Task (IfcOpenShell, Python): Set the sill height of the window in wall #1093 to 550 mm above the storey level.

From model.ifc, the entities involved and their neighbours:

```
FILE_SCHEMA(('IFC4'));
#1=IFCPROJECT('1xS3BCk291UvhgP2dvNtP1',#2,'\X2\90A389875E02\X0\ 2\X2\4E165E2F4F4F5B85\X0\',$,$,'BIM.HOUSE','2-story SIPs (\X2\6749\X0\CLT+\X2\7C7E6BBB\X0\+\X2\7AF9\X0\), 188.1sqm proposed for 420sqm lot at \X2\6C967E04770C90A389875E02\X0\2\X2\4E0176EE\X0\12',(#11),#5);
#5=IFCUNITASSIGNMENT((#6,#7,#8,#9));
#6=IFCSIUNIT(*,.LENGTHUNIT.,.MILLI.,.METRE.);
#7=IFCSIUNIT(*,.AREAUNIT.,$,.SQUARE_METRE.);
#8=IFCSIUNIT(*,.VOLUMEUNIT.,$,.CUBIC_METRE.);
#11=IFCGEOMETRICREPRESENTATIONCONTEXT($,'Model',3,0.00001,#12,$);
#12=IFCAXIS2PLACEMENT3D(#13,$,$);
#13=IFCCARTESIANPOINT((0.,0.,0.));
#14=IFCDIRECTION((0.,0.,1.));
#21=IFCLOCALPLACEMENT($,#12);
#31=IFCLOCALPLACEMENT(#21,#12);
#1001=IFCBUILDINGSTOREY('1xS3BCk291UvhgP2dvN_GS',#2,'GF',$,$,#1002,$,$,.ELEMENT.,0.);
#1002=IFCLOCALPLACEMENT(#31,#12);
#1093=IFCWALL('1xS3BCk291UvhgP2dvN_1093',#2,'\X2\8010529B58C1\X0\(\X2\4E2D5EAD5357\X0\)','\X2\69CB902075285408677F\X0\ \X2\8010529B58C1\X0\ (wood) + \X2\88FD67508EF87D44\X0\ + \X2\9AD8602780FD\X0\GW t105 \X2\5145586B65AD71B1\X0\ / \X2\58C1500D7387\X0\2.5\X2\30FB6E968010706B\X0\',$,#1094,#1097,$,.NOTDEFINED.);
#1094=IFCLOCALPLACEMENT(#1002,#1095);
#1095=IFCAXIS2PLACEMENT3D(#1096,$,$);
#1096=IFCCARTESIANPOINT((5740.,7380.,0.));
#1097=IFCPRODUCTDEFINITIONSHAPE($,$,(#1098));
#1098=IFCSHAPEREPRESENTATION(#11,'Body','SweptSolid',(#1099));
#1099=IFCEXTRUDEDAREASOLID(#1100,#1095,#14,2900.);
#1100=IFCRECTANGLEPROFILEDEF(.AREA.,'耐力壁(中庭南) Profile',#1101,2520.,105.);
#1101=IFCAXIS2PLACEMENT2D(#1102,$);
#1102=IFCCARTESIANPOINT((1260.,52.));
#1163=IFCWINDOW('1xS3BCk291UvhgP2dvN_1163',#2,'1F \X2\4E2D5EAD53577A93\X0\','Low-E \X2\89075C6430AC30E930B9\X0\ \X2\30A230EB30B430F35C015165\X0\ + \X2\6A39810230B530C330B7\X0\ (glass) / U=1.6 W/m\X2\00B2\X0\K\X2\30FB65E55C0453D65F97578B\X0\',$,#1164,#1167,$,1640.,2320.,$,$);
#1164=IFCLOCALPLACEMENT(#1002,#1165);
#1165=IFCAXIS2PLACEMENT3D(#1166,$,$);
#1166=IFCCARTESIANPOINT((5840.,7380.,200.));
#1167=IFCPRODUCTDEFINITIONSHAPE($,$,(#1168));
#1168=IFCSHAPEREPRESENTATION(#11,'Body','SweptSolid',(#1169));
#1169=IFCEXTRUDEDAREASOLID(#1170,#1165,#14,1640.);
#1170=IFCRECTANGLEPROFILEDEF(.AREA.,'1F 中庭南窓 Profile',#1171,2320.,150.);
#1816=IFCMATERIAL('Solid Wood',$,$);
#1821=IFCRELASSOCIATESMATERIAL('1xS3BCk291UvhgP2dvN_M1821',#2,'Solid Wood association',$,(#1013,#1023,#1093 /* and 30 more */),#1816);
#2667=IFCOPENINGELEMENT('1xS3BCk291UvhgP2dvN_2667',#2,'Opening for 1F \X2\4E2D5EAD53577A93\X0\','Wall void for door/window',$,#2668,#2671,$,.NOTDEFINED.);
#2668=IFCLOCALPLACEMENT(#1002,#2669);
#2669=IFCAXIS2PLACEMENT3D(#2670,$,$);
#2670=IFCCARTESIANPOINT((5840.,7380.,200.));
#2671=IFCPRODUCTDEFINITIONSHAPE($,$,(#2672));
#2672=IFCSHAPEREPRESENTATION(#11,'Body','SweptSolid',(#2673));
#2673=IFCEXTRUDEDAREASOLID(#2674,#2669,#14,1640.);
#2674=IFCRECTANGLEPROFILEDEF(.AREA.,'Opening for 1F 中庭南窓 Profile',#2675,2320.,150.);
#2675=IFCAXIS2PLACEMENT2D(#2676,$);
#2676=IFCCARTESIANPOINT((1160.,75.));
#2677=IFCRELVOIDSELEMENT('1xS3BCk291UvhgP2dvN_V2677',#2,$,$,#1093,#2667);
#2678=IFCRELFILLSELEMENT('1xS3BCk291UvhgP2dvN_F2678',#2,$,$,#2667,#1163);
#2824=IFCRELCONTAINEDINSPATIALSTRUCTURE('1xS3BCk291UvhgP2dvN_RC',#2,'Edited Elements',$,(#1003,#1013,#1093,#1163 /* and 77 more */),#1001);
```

```python
import numpy as np
import ifcopenshell
import ifcopenshell.api.geometry
import ifcopenshell.geom
import ifcopenshell.util.element
import ifcopenshell.util.placement
import ifcopenshell.util.shape
import ifcopenshell.util.unit

model = ifcopenshell.open("model.ifc")
unit_scale = ifcopenshell.util.unit.calculate_unit_scale(model)

window = model.by_guid("1xS3BCk291UvhgP2dvN_1163")
opening = window.FillsVoids[0].RelatingOpeningElement
storey = ifcopenshell.util.element.get_container(window, ifc_class="IfcBuildingStorey")
level = ifcopenshell.util.placement.get_local_placement(storey.ObjectPlacement)[2, 3]

# The opening's origin need not be at the sill, so measure its lowest point.
shape = ifcopenshell.geom.create_shape(ifcopenshell.geom.settings(), opening)
bottom = ifcopenshell.util.shape.get_shape_bottom_elevation(shape, shape.geometry) / unit_scale
dz = level + 0.55 / unit_scale - bottom

shift = np.array([0.0, 0.0, dz])
# The window is not placed relative to its opening, so move both.
for product in (opening, window):
    matrix = ifcopenshell.util.placement.get_local_placement(product.ObjectPlacement)
    matrix[:3, 3] += shift
    ifcopenshell.api.geometry.edit_object_placement(model, product=product, matrix=matrix, is_si=False)

print(f"moved by {dz * unit_scale:+.3f} m")

model.write("model_edited.ifc")
```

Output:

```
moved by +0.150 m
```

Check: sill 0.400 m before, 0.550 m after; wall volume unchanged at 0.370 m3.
